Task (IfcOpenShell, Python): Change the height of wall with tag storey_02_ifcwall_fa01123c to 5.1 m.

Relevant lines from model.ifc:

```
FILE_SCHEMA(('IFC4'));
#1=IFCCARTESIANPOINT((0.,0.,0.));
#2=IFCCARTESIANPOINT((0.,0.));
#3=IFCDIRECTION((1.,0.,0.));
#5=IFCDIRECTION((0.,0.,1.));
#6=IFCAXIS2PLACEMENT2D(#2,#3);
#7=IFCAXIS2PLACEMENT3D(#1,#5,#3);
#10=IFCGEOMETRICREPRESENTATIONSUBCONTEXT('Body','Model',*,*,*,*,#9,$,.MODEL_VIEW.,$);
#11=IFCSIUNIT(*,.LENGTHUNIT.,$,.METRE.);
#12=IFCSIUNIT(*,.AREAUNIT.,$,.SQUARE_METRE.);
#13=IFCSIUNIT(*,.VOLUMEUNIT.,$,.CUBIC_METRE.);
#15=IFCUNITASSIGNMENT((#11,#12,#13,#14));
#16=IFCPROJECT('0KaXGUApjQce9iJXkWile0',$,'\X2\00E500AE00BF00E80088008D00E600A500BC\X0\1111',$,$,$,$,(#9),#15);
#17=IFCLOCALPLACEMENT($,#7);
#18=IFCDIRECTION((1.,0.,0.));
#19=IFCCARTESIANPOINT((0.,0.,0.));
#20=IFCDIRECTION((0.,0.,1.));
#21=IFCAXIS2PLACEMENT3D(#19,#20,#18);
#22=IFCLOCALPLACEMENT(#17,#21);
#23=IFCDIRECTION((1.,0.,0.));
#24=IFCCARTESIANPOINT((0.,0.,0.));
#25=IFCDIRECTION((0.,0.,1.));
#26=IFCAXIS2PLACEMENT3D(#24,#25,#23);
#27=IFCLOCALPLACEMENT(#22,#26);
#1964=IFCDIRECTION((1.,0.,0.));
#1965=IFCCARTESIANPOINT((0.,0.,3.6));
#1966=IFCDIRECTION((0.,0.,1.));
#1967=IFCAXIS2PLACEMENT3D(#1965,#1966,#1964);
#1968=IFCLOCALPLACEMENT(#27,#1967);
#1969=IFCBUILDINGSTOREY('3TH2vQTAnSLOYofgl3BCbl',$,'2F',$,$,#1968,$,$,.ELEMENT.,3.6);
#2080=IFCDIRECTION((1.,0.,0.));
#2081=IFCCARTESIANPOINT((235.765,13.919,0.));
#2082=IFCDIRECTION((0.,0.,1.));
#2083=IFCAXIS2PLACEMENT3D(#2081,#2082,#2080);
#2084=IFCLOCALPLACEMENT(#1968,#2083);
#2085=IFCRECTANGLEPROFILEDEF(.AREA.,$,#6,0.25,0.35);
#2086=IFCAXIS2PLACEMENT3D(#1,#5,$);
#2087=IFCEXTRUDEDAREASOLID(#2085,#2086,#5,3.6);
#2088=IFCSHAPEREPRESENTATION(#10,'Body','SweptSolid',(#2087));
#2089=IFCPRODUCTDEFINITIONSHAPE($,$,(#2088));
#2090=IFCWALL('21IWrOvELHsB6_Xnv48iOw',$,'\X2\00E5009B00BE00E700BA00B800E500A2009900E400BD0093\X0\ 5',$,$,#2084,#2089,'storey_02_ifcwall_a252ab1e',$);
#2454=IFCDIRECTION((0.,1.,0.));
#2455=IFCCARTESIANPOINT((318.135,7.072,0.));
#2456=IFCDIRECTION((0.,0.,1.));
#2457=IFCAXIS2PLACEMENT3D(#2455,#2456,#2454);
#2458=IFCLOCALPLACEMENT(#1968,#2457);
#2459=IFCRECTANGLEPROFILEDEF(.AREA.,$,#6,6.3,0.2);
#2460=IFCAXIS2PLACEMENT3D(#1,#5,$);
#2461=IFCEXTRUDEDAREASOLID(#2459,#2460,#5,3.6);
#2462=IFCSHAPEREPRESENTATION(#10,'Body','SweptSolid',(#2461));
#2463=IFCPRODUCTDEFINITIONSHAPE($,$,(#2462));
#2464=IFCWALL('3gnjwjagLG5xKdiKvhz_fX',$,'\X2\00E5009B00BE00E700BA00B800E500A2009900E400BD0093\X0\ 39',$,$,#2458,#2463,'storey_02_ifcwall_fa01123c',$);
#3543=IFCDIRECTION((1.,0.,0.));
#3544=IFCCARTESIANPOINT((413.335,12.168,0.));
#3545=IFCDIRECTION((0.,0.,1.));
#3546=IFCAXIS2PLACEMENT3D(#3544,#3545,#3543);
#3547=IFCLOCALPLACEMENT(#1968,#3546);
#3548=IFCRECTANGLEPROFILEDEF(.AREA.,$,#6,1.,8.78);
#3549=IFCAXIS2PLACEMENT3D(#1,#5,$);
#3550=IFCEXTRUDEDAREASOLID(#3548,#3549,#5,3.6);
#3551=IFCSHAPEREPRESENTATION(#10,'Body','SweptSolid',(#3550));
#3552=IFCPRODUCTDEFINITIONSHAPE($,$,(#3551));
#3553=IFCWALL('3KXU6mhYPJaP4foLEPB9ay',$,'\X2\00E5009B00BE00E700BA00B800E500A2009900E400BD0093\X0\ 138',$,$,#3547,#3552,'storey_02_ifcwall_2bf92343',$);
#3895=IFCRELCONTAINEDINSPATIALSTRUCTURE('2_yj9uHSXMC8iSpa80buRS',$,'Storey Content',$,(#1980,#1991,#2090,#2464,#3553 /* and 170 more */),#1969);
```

```python
import ifcopenshell
import ifcopenshell.geom
import ifcopenshell.util.representation
import ifcopenshell.util.shape
import ifcopenshell.util.unit

model = ifcopenshell.open("model.ifc")
unit_scale = ifcopenshell.util.unit.calculate_unit_scale(model)
settings = ifcopenshell.geom.settings()


def volume(element):
    """Net volume in cubic metres, openings subtracted."""
    shape = ifcopenshell.geom.create_shape(settings, element)
    return ifcopenshell.util.shape.get_volume(shape.geometry)


wall = model.by_guid("3gnjwjagLG5xKdiKvhz_fX")
before = volume(wall)

body = ifcopenshell.util.representation.get_representation(wall, "Model", "Body")
solid = body.Items[0]
old_height = solid.Depth
solid.Depth = 5.1 / unit_scale
after = volume(wall)

print(f"height {old_height:g} -> {solid.Depth:g}, volume {before:.3f} -> {after:.3f} m3")

model.write("model_v2.ifc")
```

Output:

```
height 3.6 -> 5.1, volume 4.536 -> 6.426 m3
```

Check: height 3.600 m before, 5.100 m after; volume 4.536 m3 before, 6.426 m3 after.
